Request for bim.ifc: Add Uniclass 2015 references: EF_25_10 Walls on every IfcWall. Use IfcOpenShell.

First a look at what the model holds.

```python
import ifcopenshell

model = ifcopenshell.open("bim.ifc")
print(model.schema)
print("classifications:", [c.Name for c in model.by_type("IfcClassification")])
for ifc_class in ("IfcDoor", "IfcRoof", "IfcStair", "IfcWall", "IfcWindow"):
    print(ifc_class, len(model.by_type(ifc_class)))
```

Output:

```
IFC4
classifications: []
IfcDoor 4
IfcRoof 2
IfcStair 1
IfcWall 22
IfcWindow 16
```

```python
import ifcopenshell
import ifcopenshell.api.classification

model = ifcopenshell.open("bim.ifc")

system = ifcopenshell.api.classification.add_classification(model, classification="Uniclass 2015")

codes = {
    "IfcWall": ("EF_25_10", "Walls"),
}
for ifc_class, (code, name) in codes.items():
    products = model.by_type(ifc_class)
    ifcopenshell.api.classification.add_reference(
        model, products=products, classification=system, identification=code, name=name
    )
    print(code, len(products))

model.write("bim_updated.ifc")
```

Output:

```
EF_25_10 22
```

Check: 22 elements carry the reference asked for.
